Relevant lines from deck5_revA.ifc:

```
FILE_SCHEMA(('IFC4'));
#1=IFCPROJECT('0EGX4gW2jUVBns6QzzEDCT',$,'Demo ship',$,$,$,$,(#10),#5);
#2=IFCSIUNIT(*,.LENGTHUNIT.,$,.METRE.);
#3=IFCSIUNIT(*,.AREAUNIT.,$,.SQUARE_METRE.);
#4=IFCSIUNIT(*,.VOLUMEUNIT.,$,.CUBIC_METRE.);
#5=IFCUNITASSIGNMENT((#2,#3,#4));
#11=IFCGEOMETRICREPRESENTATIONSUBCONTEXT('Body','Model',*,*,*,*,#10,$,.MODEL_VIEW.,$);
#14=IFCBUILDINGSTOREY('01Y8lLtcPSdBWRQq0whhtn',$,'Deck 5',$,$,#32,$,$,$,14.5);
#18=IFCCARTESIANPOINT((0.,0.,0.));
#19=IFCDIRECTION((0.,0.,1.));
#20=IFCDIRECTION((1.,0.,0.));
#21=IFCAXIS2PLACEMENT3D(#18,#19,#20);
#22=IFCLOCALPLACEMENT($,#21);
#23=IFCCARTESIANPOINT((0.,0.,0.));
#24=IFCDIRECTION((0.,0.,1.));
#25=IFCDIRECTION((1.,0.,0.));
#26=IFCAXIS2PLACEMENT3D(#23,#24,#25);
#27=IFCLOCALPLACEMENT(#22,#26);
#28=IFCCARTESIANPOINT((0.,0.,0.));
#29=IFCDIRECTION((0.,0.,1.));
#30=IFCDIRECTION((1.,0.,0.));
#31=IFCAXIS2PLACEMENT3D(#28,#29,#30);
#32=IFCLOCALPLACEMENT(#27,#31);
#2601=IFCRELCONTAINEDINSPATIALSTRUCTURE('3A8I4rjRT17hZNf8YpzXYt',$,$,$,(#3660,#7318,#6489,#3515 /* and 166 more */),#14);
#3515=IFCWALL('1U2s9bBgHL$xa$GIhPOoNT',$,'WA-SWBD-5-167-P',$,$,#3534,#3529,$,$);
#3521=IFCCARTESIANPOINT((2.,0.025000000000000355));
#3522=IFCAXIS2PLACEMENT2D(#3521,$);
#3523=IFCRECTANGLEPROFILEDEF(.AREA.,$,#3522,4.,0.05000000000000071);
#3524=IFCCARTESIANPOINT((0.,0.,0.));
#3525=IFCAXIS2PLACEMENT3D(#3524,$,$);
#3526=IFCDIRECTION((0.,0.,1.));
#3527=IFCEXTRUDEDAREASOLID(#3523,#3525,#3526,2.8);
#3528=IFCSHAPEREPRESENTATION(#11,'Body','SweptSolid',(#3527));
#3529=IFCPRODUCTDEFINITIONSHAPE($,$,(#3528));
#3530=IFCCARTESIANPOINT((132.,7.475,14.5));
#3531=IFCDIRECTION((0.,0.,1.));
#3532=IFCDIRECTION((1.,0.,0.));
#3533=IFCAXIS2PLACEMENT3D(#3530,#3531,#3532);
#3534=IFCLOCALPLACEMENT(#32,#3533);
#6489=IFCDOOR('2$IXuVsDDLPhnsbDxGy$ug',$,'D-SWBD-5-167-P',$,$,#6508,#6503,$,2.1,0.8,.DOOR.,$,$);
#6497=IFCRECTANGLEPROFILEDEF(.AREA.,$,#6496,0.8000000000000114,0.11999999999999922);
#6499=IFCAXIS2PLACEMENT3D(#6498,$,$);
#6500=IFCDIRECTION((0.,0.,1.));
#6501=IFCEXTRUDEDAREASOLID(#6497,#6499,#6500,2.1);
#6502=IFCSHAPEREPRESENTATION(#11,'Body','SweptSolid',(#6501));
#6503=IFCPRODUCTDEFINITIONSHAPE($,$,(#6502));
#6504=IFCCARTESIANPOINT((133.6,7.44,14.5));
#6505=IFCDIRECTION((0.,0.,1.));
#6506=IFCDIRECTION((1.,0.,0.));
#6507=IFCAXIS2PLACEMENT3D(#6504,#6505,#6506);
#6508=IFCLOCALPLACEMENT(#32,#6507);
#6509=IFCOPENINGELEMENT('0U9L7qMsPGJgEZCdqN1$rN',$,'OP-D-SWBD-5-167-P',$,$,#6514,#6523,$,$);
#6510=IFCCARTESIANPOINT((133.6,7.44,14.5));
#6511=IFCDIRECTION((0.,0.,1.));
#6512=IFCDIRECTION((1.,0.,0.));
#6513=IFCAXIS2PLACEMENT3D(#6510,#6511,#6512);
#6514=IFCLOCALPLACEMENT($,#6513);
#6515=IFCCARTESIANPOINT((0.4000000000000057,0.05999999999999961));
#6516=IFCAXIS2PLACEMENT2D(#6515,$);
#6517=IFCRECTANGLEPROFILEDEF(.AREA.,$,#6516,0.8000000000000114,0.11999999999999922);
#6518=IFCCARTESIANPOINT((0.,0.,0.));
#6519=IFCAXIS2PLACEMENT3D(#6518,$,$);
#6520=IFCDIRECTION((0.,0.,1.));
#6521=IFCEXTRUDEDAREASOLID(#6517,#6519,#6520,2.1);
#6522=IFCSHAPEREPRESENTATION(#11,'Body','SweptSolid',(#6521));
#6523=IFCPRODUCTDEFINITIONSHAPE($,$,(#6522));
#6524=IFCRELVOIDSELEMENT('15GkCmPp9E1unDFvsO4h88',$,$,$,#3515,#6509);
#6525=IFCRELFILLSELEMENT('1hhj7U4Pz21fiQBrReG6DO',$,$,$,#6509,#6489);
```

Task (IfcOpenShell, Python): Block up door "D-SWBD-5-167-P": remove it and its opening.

```python
import ifcopenshell
import ifcopenshell.api.feature
import ifcopenshell.api.root
import ifcopenshell.geom
import ifcopenshell.util.shape

model = ifcopenshell.open("deck5_revA.ifc")
settings = ifcopenshell.geom.settings()


def volume(element):
    """Net volume in cubic metres, openings subtracted."""
    shape = ifcopenshell.geom.create_shape(settings, element)
    return ifcopenshell.util.shape.get_volume(shape.geometry)


door = model.by_id(6489)
opening = door.FillsVoids[0].RelatingOpeningElement
wall = opening.VoidsElements[0].RelatingBuildingElement
before = volume(wall)

ifcopenshell.api.root.remove_product(model, product=door)
ifcopenshell.api.feature.remove_feature(model, feature=opening)

after = volume(wall)

print(f"wall volume {before:.3f} -> {after:.3f} m3")

model.write("deck5_revA_rev.ifc")
```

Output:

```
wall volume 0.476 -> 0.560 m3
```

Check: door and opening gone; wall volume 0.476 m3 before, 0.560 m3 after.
